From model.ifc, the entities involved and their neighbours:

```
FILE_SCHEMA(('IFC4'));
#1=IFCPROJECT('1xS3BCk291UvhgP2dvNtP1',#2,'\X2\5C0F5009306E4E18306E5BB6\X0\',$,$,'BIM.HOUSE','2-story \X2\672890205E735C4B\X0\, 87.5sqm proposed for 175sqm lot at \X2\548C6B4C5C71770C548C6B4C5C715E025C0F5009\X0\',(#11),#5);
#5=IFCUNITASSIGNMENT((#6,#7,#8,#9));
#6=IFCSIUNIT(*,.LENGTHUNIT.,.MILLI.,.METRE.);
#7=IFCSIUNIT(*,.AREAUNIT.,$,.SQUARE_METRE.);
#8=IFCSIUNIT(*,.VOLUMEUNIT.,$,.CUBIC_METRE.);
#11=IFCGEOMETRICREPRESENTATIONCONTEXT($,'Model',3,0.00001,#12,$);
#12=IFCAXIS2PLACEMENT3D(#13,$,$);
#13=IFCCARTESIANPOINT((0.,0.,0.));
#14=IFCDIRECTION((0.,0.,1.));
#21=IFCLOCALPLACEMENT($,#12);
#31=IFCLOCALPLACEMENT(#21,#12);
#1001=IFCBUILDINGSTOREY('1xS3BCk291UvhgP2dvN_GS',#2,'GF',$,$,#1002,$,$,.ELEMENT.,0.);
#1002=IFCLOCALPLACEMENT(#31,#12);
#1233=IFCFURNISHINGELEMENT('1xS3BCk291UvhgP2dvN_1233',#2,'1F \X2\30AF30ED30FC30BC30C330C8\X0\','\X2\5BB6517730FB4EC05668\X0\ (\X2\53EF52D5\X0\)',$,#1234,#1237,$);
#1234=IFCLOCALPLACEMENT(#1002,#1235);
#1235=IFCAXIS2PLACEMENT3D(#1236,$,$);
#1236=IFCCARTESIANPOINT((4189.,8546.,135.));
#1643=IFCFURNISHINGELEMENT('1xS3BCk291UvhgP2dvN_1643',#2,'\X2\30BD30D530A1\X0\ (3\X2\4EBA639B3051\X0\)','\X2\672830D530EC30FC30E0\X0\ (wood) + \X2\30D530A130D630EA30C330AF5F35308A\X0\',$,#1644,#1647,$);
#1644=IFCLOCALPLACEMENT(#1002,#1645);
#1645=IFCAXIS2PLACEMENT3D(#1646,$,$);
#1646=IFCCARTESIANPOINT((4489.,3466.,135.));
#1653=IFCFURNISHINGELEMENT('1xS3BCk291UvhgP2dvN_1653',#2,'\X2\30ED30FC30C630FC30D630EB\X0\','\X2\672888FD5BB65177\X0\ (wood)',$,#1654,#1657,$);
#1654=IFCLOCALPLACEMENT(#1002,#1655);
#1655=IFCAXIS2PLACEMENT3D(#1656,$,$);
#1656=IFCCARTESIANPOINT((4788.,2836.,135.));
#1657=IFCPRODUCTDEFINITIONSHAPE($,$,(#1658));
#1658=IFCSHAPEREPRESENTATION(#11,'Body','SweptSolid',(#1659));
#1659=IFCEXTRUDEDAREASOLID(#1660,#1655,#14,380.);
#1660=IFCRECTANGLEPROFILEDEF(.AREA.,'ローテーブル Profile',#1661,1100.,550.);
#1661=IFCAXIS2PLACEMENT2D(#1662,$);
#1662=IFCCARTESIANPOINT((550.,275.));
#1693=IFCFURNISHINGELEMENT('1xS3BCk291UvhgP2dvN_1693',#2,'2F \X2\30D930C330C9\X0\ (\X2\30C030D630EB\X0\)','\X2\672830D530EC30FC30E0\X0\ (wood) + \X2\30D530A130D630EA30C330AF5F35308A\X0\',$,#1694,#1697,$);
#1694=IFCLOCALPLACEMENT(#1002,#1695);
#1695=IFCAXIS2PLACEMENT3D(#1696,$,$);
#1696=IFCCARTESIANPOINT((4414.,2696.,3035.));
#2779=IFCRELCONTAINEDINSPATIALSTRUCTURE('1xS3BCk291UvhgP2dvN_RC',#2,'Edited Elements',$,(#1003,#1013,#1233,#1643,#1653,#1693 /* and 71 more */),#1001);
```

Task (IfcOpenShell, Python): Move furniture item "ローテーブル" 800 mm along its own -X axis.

```python
import ifcopenshell
import ifcopenshell.api.geometry
import ifcopenshell.util.placement

model = ifcopenshell.open("model.ifc")

item = model.by_guid("1xS3BCk291UvhgP2dvN_1653")
matrix = ifcopenshell.util.placement.get_local_placement(item.ObjectPlacement)
matrix[:3, 3] -= matrix[:3, 0] * 800.0
ifcopenshell.api.geometry.edit_object_placement(model, product=item, matrix=matrix, is_si=False)

print(ifcopenshell.util.placement.get_local_placement(item.ObjectPlacement).round(3) + 0.0)

model.write("model_updated.ifc")
```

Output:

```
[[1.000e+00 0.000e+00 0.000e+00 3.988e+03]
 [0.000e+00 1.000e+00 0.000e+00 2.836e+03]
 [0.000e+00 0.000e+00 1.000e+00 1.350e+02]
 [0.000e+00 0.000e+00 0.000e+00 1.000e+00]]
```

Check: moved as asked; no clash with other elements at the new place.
